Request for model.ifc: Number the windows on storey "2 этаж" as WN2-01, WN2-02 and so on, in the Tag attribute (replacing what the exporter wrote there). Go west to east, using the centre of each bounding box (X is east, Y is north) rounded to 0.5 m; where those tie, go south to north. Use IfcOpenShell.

First a look at what the model holds.

```python
import ifcopenshell
import ifcopenshell.util.element
import ifcopenshell.util.placement

model = ifcopenshell.open("model.ifc")
print(model.schema)
storey = next(s for s in model.by_type("IfcBuildingStorey") if s.Name == "2 этаж")
windows = [e for e in ifcopenshell.util.element.get_decomposition(storey) if e.is_a("IfcWindow")]
for e in sorted(windows, key=lambda e: e.id()):
    origin = ifcopenshell.util.placement.get_local_placement(e.ObjectPlacement)[:3, 3]
    print(e.id(), e.Tag, e.Name, origin.round(2) + 0.0, sep=" | ")
```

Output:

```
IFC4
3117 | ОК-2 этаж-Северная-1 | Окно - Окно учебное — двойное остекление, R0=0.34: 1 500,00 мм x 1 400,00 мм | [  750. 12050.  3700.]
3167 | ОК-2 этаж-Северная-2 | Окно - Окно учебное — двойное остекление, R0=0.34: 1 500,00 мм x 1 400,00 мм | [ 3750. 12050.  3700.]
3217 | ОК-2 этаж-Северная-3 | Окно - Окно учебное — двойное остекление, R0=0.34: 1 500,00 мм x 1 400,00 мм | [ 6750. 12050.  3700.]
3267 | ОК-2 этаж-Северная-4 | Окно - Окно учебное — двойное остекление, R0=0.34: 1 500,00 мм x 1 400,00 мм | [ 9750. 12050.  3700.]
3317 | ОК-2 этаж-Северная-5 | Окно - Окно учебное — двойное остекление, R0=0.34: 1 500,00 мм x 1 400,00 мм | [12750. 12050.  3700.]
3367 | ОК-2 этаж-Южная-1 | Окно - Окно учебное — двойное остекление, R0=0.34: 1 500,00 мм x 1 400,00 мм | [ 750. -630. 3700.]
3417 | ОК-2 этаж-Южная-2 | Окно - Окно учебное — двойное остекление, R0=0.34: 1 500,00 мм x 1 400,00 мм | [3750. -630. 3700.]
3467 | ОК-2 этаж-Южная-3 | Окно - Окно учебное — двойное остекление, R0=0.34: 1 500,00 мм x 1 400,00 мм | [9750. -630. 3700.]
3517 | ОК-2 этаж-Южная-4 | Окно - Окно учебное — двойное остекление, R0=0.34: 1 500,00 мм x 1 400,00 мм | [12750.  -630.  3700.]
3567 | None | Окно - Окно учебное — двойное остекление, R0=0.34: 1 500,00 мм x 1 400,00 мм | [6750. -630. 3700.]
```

```python
import ifcopenshell
import ifcopenshell.geom
import ifcopenshell.util.element
import ifcopenshell.util.shape

model = ifcopenshell.open("model.ifc")
settings = ifcopenshell.geom.settings()
settings.set("use-world-coords", True)


def centre(element):
    shape = ifcopenshell.geom.create_shape(settings, element)
    return ifcopenshell.util.shape.get_bbox_centroid(shape.geometry)


storey = next(s for s in model.by_type("IfcBuildingStorey") if s.Name == "2 этаж")
windows = [e for e in ifcopenshell.util.element.get_decomposition(storey) if e.is_a("IfcWindow")]

# Insertion points can sit at a corner or the storey origin, so sort by the geometry (in metres).
centres = {e: centre(e) for e in windows}
windows.sort(key=lambda e: (round(centres[e][0] / 0.5), centres[e][1]))

for i, e in enumerate(windows, start=1):
    number = f"WN2-{i:02d}"
    e.Tag = number
    print(e.id(), number)

model.write("model_updated.ifc")
```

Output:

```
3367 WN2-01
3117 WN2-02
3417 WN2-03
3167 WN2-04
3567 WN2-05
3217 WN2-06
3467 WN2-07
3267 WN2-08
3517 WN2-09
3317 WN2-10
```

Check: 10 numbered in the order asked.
